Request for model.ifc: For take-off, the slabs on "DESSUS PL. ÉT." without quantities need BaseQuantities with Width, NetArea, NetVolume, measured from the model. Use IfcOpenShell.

First a look at what the model holds.

```python
import ifcopenshell
import ifcopenshell.util.element
import ifcopenshell.util.unit

model = ifcopenshell.open("model.ifc")
print(model.schema)
for unit_type in ("LENGTHUNIT", "AREAUNIT", "VOLUMEUNIT"):
    print(unit_type, ifcopenshell.util.unit.calculate_unit_scale(model, unit_type))
storey = next(s for s in model.by_type("IfcBuildingStorey") if s.Name == "DESSUS PL. ÉT.")
slabs = [e for e in ifcopenshell.util.element.get_decomposition(storey) if e.is_a("IfcSlab")]
for e in sorted(slabs, key=lambda e: e.id()):
    print(e.id(), e.is_a(), e.Name, list(ifcopenshell.util.element.get_psets(e, qtos_only=True)), sep=" | ")
```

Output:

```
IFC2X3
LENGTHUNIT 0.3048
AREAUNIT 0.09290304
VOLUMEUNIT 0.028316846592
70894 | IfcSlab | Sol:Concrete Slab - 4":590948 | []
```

```python
import ifcopenshell
import ifcopenshell.api.pset
import ifcopenshell.geom
import ifcopenshell.util.element
import ifcopenshell.util.shape
import ifcopenshell.util.unit

model = ifcopenshell.open("model.ifc")
unit_scale = ifcopenshell.util.unit.calculate_unit_scale(model)
area_scale = ifcopenshell.util.unit.calculate_unit_scale(model, "AREAUNIT")
volume_scale = ifcopenshell.util.unit.calculate_unit_scale(model, "VOLUMEUNIT")
settings = ifcopenshell.geom.settings()

storey = next(s for s in model.by_type("IfcBuildingStorey") if s.Name == "DESSUS PL. ÉT.")
slabs = [e for e in ifcopenshell.util.element.get_decomposition(storey) if e.is_a("IfcSlab")]

for e in sorted(slabs, key=lambda e: e.id()):
    if ifcopenshell.util.element.get_psets(e, qtos_only=True, should_inherit=False):
        continue
    # Geometry comes back in metres, in the element's own axes.
    shape = ifcopenshell.geom.create_shape(settings, e)
    values = {
        "Width": ifcopenshell.util.shape.get_z(shape.geometry) / unit_scale,
        "NetArea": ifcopenshell.util.shape.get_footprint_area(shape.geometry) / area_scale,
        "NetVolume": ifcopenshell.util.shape.get_volume(shape.geometry) / volume_scale,
    }
    qto = ifcopenshell.api.pset.add_qto(model, product=e, name="BaseQuantities")
    ifcopenshell.api.pset.edit_qto(model, qto=qto, properties=values)
    print(e.id(), {k: round(v, 3) for k, v in values.items()})

model.write("model_edited.ifc")
```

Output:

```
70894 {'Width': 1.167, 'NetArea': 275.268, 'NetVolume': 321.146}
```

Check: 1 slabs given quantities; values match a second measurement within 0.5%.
